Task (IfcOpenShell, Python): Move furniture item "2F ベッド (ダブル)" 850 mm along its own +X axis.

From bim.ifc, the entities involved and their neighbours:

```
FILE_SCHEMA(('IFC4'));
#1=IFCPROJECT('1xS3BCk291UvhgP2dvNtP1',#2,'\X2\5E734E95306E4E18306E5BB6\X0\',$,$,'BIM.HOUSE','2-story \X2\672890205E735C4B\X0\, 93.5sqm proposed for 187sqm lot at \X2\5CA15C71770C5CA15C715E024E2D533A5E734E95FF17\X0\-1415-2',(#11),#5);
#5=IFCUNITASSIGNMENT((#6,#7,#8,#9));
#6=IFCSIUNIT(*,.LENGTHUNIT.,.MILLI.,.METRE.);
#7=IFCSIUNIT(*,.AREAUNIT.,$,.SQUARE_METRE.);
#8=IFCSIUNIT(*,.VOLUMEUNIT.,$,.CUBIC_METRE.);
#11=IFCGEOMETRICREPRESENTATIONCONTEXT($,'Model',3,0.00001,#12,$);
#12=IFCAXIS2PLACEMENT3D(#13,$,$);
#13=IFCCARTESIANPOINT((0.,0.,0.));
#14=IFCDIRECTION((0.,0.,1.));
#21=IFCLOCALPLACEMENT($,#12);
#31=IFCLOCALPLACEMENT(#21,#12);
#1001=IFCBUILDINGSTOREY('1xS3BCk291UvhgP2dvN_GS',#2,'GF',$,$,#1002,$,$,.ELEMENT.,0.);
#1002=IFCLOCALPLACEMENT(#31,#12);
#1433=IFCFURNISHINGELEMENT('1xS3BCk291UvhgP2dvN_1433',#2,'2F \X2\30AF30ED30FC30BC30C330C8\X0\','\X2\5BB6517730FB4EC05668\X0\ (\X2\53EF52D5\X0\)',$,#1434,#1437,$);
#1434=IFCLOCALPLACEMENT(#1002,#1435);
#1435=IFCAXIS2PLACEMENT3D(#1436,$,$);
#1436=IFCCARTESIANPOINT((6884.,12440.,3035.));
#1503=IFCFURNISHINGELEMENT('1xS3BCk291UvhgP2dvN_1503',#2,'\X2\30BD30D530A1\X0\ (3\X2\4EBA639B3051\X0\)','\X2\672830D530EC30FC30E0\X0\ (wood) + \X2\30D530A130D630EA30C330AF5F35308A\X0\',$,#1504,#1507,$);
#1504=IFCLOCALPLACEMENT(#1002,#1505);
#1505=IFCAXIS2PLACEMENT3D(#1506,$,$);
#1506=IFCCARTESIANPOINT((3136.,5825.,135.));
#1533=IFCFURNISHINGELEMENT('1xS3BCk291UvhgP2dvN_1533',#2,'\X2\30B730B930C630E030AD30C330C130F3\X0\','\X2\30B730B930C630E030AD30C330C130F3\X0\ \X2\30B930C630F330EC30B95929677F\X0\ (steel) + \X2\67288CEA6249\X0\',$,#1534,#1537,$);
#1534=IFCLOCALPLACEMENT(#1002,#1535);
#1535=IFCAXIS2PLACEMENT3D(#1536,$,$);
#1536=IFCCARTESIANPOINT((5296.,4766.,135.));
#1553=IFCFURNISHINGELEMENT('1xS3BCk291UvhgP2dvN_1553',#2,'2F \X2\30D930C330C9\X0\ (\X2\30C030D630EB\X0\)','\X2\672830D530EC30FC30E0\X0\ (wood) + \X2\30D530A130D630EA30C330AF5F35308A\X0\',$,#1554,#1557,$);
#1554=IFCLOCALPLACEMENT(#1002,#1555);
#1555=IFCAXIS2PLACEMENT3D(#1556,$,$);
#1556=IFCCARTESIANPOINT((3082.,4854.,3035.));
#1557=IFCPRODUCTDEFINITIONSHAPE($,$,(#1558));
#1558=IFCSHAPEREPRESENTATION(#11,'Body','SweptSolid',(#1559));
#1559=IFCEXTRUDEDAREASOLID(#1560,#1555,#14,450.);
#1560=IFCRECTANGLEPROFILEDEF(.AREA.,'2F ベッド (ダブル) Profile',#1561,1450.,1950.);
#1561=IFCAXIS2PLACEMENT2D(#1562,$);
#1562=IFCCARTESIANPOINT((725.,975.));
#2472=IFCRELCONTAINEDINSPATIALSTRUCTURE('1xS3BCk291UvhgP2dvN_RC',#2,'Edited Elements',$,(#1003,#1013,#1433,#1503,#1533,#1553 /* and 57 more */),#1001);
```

```python
import ifcopenshell
import ifcopenshell.api.geometry
import ifcopenshell.util.placement

model = ifcopenshell.open("bim.ifc")

item = model.by_guid("1xS3BCk291UvhgP2dvN_1553")
matrix = ifcopenshell.util.placement.get_local_placement(item.ObjectPlacement)
matrix[:3, 3] += matrix[:3, 0] * 850.0
ifcopenshell.api.geometry.edit_object_placement(model, product=item, matrix=matrix, is_si=False)

print(ifcopenshell.util.placement.get_local_placement(item.ObjectPlacement).round(3) + 0.0)

model.write("bim_v2.ifc")
```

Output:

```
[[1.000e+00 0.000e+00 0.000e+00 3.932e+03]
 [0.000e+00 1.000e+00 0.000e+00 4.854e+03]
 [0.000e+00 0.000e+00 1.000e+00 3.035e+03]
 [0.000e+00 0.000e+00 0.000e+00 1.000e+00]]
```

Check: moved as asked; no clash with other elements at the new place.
